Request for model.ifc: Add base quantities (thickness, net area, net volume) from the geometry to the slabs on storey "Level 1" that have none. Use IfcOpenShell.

First a look at what the model holds.

```python
import ifcopenshell
import ifcopenshell.util.element
import ifcopenshell.util.unit

model = ifcopenshell.open("model.ifc")
print(model.schema)
for unit_type in ("LENGTHUNIT", "AREAUNIT", "VOLUMEUNIT"):
    print(unit_type, ifcopenshell.util.unit.calculate_unit_scale(model, unit_type))
storey = next(s for s in model.by_type("IfcBuildingStorey") if s.Name == "Level 1")
slabs = [e for e in ifcopenshell.util.element.get_decomposition(storey) if e.is_a("IfcSlab")]
for e in sorted(slabs, key=lambda e: e.id()):
    print(e.id(), e.is_a(), e.Name, list(ifcopenshell.util.element.get_psets(e, qtos_only=True)), sep=" | ")
```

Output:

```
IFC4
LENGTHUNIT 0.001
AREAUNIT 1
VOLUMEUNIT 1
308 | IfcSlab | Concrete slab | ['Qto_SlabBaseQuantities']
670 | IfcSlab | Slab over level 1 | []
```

```python
import ifcopenshell
import ifcopenshell.api.pset
import ifcopenshell.geom
import ifcopenshell.util.element
import ifcopenshell.util.shape
import ifcopenshell.util.unit

model = ifcopenshell.open("model.ifc")
unit_scale = ifcopenshell.util.unit.calculate_unit_scale(model)
area_scale = ifcopenshell.util.unit.calculate_unit_scale(model, "AREAUNIT")
volume_scale = ifcopenshell.util.unit.calculate_unit_scale(model, "VOLUMEUNIT")
settings = ifcopenshell.geom.settings()

storey = next(s for s in model.by_type("IfcBuildingStorey") if s.Name == "Level 1")
slabs = [e for e in ifcopenshell.util.element.get_decomposition(storey) if e.is_a("IfcSlab")]

for e in sorted(slabs, key=lambda e: e.id()):
    if ifcopenshell.util.element.get_psets(e, qtos_only=True, should_inherit=False):
        continue
    # Geometry comes back in metres, in the element's own axes.
    shape = ifcopenshell.geom.create_shape(settings, e)
    values = {
        "Width": ifcopenshell.util.shape.get_z(shape.geometry) / unit_scale,
        "NetArea": ifcopenshell.util.shape.get_footprint_area(shape.geometry) / area_scale,
        "NetVolume": ifcopenshell.util.shape.get_volume(shape.geometry) / volume_scale,
    }
    qto = ifcopenshell.api.pset.add_qto(model, product=e, name="Qto_SlabBaseQuantities")
    ifcopenshell.api.pset.edit_qto(model, qto=qto, properties=values)
    print(e.id(), {k: round(v, 3) for k, v in values.items()})

model.write("model_edited.ifc")
```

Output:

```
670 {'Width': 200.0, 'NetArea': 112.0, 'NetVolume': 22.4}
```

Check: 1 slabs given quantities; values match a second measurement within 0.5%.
